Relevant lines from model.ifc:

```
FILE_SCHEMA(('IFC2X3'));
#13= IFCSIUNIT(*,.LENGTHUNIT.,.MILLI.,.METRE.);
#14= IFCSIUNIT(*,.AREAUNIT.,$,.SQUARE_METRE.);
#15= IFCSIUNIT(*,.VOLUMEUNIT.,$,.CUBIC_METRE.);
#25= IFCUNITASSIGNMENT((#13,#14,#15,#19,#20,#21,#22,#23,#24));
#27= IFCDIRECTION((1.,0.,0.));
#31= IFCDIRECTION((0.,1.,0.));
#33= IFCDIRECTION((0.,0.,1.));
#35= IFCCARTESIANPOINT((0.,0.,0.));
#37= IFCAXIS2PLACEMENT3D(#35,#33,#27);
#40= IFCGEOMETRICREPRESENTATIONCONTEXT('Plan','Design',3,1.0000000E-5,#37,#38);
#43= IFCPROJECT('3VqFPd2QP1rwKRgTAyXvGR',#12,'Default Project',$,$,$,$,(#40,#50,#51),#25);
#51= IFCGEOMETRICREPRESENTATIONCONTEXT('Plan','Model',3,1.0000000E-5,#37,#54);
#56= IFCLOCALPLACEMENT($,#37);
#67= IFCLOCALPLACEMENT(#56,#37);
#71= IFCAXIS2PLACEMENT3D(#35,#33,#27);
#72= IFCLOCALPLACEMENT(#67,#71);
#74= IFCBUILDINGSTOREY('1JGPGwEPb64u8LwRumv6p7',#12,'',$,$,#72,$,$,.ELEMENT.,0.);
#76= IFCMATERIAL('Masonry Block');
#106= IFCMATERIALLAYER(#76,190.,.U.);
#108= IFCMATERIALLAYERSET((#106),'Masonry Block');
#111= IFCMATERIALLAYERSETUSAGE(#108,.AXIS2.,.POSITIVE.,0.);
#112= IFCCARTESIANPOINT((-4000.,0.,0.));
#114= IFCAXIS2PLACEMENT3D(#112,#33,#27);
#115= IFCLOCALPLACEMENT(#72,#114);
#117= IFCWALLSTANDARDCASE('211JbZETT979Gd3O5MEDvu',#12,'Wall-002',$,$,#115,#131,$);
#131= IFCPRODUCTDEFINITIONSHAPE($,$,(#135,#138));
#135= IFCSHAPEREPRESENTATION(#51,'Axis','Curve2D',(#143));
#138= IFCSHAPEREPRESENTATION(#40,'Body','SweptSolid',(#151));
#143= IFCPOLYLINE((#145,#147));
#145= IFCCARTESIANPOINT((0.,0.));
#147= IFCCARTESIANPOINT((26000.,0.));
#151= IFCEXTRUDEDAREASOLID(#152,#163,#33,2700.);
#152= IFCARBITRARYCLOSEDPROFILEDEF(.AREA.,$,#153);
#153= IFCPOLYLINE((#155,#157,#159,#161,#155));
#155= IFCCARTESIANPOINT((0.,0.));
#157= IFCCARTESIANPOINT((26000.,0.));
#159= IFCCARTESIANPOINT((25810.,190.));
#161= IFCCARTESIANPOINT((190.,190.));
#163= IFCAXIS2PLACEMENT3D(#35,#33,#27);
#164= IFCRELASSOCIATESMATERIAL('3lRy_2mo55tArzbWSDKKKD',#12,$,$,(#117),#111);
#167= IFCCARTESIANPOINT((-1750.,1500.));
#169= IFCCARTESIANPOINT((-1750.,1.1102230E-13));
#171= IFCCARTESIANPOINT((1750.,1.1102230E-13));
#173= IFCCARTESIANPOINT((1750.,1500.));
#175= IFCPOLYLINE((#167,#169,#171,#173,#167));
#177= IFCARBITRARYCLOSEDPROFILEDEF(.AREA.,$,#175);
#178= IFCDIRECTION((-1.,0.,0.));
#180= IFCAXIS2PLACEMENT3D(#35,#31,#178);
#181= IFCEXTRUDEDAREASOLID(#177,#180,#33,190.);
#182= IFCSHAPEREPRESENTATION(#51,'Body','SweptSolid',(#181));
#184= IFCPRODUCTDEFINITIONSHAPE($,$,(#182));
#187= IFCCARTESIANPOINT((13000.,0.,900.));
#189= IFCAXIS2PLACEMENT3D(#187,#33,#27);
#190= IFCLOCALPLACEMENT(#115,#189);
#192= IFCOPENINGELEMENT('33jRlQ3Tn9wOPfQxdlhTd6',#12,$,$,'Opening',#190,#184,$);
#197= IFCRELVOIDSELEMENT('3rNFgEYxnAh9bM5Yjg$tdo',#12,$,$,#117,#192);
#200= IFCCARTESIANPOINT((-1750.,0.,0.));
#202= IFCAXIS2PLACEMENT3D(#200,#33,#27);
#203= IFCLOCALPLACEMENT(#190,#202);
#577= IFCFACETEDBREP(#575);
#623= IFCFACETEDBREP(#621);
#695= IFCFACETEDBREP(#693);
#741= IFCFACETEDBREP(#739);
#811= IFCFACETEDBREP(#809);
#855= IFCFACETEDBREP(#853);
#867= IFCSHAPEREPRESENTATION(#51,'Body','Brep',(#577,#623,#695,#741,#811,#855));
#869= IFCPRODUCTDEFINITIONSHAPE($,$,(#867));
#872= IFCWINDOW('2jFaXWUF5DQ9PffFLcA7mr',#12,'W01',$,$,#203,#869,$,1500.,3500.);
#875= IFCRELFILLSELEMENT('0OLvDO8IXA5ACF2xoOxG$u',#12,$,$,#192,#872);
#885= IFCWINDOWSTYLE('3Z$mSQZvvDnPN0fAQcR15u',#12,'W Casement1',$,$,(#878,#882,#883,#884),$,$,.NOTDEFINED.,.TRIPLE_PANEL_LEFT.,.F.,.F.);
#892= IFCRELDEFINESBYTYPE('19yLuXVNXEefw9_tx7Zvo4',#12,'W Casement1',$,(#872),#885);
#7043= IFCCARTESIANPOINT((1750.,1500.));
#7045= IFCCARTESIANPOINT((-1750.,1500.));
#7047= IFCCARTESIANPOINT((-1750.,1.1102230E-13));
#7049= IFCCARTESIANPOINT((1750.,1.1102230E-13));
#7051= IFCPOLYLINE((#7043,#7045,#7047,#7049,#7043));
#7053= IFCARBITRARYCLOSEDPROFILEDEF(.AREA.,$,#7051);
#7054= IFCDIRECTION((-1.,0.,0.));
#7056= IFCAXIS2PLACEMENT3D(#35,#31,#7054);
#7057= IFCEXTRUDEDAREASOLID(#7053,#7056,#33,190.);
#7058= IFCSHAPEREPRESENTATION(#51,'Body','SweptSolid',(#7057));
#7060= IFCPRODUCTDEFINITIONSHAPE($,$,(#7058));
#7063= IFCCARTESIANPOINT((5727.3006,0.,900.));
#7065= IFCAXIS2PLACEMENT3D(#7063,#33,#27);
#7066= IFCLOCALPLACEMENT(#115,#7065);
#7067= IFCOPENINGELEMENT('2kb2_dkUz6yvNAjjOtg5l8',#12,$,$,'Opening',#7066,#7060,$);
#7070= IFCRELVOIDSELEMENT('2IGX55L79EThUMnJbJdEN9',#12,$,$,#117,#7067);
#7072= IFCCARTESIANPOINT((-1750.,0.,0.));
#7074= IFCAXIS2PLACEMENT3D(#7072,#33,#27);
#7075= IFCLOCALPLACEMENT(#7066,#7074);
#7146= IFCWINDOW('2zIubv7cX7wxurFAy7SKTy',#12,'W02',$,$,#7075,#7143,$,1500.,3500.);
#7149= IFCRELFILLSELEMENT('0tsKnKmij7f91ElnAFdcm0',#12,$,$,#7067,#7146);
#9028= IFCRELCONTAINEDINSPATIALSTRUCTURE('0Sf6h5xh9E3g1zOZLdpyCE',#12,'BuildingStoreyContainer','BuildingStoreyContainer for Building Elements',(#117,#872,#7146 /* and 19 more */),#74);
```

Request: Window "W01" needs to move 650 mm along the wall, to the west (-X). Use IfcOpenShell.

```python
import ifcopenshell
import ifcopenshell.api.geometry
import ifcopenshell.util.placement

model = ifcopenshell.open("model.ifc")

window = model.by_guid("2jFaXWUF5DQ9PffFLcA7mr")
opening = window.FillsVoids[0].RelatingOpeningElement
wall = opening.VoidsElements[0].RelatingBuildingElement

wall_matrix = ifcopenshell.util.placement.get_local_placement(wall.ObjectPlacement)
shift = wall_matrix[:3, 0] * -650.0
before = ifcopenshell.util.placement.get_local_placement(window.ObjectPlacement)[:3, 3].copy()

# The window is placed relative to its opening, so it follows when the opening moves.
matrix = ifcopenshell.util.placement.get_local_placement(opening.ObjectPlacement)
matrix[:3, 3] += shift
ifcopenshell.api.geometry.edit_object_placement(
    model, product=opening, matrix=matrix, is_si=False, should_transform_children=True
)

after = ifcopenshell.util.placement.get_local_placement(window.ObjectPlacement)[:3, 3]
print("window moved by", (after - before).round(3) + 0.0)

model.write("model_edited.ifc")
```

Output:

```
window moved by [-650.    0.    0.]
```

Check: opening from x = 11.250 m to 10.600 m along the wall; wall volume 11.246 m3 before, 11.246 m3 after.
